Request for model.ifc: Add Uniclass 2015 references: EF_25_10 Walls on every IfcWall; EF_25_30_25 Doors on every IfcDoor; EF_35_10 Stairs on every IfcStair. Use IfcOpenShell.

First a look at what the model holds.

```python
import ifcopenshell

model = ifcopenshell.open("model.ifc")
print(model.schema)
print("classifications:", [c.Name for c in model.by_type("IfcClassification")])
for ifc_class in ("IfcDoor", "IfcRoof", "IfcStair", "IfcWall", "IfcWindow"):
    print(ifc_class, len(model.by_type(ifc_class)))
```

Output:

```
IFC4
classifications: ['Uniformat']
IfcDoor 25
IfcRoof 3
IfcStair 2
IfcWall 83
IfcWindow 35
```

```python
import ifcopenshell
import ifcopenshell.api.classification

model = ifcopenshell.open("model.ifc")

system = ifcopenshell.api.classification.add_classification(model, classification="Uniclass 2015")

codes = {
    "IfcWall": ("EF_25_10", "Walls"),
    "IfcDoor": ("EF_25_30_25", "Doors"),
    "IfcStair": ("EF_35_10", "Stairs"),
}
for ifc_class, (code, name) in codes.items():
    products = model.by_type(ifc_class)
    ifcopenshell.api.classification.add_reference(
        model, products=products, classification=system, identification=code, name=name
    )
    print(code, len(products))

model.write("model_updated.ifc")
```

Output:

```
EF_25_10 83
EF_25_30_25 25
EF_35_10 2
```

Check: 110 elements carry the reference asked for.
